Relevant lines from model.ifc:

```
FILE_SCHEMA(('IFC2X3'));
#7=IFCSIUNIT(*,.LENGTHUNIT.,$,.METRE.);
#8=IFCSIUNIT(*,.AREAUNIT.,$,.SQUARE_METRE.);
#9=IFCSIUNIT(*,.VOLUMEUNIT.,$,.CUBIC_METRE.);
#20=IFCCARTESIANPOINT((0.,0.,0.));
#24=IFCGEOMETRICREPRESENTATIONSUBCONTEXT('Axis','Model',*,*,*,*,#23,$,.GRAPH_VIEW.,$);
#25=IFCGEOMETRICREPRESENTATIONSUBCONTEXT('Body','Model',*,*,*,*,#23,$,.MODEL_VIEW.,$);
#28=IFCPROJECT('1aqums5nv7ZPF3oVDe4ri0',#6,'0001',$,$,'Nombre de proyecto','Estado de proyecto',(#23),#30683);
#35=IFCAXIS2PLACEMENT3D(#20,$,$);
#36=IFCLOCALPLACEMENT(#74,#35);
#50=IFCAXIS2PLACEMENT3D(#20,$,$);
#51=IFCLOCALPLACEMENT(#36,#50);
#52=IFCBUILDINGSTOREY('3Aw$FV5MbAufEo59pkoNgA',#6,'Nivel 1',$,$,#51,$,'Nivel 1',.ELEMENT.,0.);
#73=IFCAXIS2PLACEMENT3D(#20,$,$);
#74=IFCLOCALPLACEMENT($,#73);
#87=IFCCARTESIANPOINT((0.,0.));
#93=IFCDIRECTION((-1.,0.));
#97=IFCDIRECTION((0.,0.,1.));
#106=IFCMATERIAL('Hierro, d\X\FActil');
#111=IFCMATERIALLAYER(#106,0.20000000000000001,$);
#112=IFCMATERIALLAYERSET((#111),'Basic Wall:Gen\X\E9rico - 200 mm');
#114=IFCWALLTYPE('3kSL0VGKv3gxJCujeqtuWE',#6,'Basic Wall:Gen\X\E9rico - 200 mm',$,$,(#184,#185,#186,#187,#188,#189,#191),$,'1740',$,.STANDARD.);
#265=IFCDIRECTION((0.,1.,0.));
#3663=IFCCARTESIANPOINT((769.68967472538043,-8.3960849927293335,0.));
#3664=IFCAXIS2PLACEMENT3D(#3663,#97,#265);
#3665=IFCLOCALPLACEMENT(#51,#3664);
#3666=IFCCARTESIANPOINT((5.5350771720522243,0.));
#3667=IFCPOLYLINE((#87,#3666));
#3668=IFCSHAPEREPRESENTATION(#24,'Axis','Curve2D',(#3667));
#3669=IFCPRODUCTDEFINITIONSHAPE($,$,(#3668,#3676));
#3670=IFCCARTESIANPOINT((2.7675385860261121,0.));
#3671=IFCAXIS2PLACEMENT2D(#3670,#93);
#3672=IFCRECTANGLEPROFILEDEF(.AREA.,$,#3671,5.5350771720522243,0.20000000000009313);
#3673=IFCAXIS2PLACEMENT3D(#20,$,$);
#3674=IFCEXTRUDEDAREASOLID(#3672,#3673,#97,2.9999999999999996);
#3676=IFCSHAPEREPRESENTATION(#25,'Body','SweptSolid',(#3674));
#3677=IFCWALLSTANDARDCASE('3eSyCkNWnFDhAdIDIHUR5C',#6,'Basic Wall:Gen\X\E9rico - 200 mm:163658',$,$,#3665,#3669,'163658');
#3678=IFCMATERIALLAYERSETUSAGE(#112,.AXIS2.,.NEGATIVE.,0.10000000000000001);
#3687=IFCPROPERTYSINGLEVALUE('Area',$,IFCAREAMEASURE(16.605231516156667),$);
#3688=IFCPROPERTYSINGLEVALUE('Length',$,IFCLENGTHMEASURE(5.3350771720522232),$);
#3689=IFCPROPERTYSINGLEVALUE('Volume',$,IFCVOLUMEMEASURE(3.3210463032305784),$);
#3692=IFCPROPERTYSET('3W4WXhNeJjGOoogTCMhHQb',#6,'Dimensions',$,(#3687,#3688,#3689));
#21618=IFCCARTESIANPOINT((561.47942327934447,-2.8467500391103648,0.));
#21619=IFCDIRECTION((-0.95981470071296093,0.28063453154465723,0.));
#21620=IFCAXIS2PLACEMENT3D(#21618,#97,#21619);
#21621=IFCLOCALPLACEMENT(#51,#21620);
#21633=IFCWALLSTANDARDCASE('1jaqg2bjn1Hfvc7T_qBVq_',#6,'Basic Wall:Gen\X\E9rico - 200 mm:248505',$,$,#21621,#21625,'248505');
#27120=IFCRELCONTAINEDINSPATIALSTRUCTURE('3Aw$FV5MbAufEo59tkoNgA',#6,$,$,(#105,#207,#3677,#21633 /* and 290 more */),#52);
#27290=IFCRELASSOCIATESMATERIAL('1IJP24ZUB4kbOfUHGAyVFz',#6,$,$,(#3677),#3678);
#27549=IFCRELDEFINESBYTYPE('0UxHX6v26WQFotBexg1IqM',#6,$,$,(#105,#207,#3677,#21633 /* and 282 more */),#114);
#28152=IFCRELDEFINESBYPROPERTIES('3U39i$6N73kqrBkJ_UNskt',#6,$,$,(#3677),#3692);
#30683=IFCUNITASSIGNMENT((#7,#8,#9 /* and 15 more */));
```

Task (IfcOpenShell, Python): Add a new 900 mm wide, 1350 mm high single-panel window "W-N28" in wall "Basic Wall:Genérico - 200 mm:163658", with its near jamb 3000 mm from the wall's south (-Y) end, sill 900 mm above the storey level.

```python
import numpy as np
import ifcopenshell
import ifcopenshell.api.feature
import ifcopenshell.api.geometry
import ifcopenshell.api.pset
import ifcopenshell.api.root
import ifcopenshell.api.spatial
import ifcopenshell.api.type
import ifcopenshell.geom
import ifcopenshell.util.element
import ifcopenshell.util.placement
import ifcopenshell.util.representation
import ifcopenshell.util.shape
import ifcopenshell.util.unit

model = ifcopenshell.open("model.ifc")
unit_scale = ifcopenshell.util.unit.calculate_unit_scale(model)
area_scale = ifcopenshell.util.unit.calculate_unit_scale(model, "AREAUNIT")
volume_scale = ifcopenshell.util.unit.calculate_unit_scale(model, "VOLUMEUNIT")
settings = ifcopenshell.geom.settings()


def volume(element):
    """Net volume in cubic metres, openings subtracted."""
    shape = ifcopenshell.geom.create_shape(settings, element)
    return ifcopenshell.util.shape.get_volume(shape.geometry)


wall = model.by_guid("3eSyCkNWnFDhAdIDIHUR5C")
storey = ifcopenshell.util.element.get_container(wall, ifc_class="IfcBuildingStorey")
context = ifcopenshell.util.representation.get_context(model, "Model", "Body", "MODEL_VIEW")
before = volume(wall)

width, height, from_end, sill = 0.9, 1.35, 3, 0.9  # metres

# The wall runs along its own X axis, and the end named is its -X end.
wall_shape = ifcopenshell.geom.create_shape(settings, wall)
x, y, z = ifcopenshell.util.shape.get_vertices(wall_shape.geometry).T
start = x.min() + from_end
face, thickness = float(y.min()), float(y.max() - y.min())
wall_matrix = ifcopenshell.util.placement.get_local_placement(wall.ObjectPlacement)
level = ifcopenshell.util.placement.get_local_placement(storey.ObjectPlacement)[2, 3]


def in_wall(x, y):
    """Placement at x, y metres in the wall's axes, at sill height."""
    matrix = wall_matrix.copy()
    matrix[:, 3] = wall_matrix @ np.array([x / unit_scale, y / unit_scale, 0.0, 1.0])
    matrix[2, 3] = level + sill / unit_scale
    return matrix


# Opening: a box that overshoots both wall faces by 50 mm.
opening = ifcopenshell.api.root.create_entity(model, ifc_class="IfcOpeningElement")
box = ifcopenshell.api.geometry.add_wall_representation(
    model, context=context, length=width, height=height, thickness=thickness + 0.1
)
ifcopenshell.api.geometry.assign_representation(model, product=opening, representation=box)
ifcopenshell.api.geometry.edit_object_placement(model, product=opening, matrix=in_wall(start, face - 0.05), is_si=False)
ifcopenshell.api.feature.add_feature(model, feature=opening, element=wall)

window = ifcopenshell.api.root.create_entity(model, ifc_class="IfcWindow", name="W-N28")
window.OverallWidth, window.OverallHeight = width / unit_scale, height / unit_scale
body = ifcopenshell.api.geometry.add_window_representation(
    model,
    context=context,
    overall_width=window.OverallWidth,
    overall_height=window.OverallHeight,
    partition_type="SINGLE_PANEL",
)
ifcopenshell.api.geometry.assign_representation(model, product=window, representation=body)
ifcopenshell.api.spatial.assign_container(model, products=[window], relating_structure=storey)
fills = ifcopenshell.api.feature.add_filling(model, opening=opening, element=window)
fills.OwnerHistory = window.OwnerHistory  # required in IFC2X3

# IFC2X3 keeps the operation on the window style.
style = ifcopenshell.api.root.create_entity(model, ifc_class="IfcWindowStyle", name="W-N28")
style.OperationType, style.ConstructionType = "SINGLE_PANEL", "NOTDEFINED"
style.ParameterTakesPrecedence = style.Sizeable = False
ifcopenshell.api.type.assign_type(model, related_objects=[window], relating_type=style)

# Centre the window in the wall's thickness.
ifcopenshell.api.geometry.edit_object_placement(model, product=window, matrix=in_wall(start, face), is_si=False)
window_shape = ifcopenshell.geom.create_shape(settings, window)
depth = ifcopenshell.util.shape.get_vertices(window_shape.geometry)[:, 1]
offset = face + thickness / 2 - (depth.min() + depth.max()) / 2
ifcopenshell.api.geometry.edit_object_placement(model, product=window, matrix=in_wall(start, offset), is_si=False)

after = volume(wall)

# Update the wall's stored quantities.
pset = model.by_id(ifcopenshell.util.element.get_pset(wall, "Dimensions", should_inherit=False)["id"])
ifcopenshell.api.pset.edit_pset(model, pset=pset, properties={
    "Area": model.create_entity("IfcAreaMeasure", after / thickness / area_scale),
    "Volume": model.create_entity("IfcVolumeMeasure", after / volume_scale),
})

print(f"wall volume {before:.3f} -> {after:.3f} m3")

model.write("model_rev.ifc")
```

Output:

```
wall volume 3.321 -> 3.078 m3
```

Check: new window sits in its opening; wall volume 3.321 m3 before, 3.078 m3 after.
